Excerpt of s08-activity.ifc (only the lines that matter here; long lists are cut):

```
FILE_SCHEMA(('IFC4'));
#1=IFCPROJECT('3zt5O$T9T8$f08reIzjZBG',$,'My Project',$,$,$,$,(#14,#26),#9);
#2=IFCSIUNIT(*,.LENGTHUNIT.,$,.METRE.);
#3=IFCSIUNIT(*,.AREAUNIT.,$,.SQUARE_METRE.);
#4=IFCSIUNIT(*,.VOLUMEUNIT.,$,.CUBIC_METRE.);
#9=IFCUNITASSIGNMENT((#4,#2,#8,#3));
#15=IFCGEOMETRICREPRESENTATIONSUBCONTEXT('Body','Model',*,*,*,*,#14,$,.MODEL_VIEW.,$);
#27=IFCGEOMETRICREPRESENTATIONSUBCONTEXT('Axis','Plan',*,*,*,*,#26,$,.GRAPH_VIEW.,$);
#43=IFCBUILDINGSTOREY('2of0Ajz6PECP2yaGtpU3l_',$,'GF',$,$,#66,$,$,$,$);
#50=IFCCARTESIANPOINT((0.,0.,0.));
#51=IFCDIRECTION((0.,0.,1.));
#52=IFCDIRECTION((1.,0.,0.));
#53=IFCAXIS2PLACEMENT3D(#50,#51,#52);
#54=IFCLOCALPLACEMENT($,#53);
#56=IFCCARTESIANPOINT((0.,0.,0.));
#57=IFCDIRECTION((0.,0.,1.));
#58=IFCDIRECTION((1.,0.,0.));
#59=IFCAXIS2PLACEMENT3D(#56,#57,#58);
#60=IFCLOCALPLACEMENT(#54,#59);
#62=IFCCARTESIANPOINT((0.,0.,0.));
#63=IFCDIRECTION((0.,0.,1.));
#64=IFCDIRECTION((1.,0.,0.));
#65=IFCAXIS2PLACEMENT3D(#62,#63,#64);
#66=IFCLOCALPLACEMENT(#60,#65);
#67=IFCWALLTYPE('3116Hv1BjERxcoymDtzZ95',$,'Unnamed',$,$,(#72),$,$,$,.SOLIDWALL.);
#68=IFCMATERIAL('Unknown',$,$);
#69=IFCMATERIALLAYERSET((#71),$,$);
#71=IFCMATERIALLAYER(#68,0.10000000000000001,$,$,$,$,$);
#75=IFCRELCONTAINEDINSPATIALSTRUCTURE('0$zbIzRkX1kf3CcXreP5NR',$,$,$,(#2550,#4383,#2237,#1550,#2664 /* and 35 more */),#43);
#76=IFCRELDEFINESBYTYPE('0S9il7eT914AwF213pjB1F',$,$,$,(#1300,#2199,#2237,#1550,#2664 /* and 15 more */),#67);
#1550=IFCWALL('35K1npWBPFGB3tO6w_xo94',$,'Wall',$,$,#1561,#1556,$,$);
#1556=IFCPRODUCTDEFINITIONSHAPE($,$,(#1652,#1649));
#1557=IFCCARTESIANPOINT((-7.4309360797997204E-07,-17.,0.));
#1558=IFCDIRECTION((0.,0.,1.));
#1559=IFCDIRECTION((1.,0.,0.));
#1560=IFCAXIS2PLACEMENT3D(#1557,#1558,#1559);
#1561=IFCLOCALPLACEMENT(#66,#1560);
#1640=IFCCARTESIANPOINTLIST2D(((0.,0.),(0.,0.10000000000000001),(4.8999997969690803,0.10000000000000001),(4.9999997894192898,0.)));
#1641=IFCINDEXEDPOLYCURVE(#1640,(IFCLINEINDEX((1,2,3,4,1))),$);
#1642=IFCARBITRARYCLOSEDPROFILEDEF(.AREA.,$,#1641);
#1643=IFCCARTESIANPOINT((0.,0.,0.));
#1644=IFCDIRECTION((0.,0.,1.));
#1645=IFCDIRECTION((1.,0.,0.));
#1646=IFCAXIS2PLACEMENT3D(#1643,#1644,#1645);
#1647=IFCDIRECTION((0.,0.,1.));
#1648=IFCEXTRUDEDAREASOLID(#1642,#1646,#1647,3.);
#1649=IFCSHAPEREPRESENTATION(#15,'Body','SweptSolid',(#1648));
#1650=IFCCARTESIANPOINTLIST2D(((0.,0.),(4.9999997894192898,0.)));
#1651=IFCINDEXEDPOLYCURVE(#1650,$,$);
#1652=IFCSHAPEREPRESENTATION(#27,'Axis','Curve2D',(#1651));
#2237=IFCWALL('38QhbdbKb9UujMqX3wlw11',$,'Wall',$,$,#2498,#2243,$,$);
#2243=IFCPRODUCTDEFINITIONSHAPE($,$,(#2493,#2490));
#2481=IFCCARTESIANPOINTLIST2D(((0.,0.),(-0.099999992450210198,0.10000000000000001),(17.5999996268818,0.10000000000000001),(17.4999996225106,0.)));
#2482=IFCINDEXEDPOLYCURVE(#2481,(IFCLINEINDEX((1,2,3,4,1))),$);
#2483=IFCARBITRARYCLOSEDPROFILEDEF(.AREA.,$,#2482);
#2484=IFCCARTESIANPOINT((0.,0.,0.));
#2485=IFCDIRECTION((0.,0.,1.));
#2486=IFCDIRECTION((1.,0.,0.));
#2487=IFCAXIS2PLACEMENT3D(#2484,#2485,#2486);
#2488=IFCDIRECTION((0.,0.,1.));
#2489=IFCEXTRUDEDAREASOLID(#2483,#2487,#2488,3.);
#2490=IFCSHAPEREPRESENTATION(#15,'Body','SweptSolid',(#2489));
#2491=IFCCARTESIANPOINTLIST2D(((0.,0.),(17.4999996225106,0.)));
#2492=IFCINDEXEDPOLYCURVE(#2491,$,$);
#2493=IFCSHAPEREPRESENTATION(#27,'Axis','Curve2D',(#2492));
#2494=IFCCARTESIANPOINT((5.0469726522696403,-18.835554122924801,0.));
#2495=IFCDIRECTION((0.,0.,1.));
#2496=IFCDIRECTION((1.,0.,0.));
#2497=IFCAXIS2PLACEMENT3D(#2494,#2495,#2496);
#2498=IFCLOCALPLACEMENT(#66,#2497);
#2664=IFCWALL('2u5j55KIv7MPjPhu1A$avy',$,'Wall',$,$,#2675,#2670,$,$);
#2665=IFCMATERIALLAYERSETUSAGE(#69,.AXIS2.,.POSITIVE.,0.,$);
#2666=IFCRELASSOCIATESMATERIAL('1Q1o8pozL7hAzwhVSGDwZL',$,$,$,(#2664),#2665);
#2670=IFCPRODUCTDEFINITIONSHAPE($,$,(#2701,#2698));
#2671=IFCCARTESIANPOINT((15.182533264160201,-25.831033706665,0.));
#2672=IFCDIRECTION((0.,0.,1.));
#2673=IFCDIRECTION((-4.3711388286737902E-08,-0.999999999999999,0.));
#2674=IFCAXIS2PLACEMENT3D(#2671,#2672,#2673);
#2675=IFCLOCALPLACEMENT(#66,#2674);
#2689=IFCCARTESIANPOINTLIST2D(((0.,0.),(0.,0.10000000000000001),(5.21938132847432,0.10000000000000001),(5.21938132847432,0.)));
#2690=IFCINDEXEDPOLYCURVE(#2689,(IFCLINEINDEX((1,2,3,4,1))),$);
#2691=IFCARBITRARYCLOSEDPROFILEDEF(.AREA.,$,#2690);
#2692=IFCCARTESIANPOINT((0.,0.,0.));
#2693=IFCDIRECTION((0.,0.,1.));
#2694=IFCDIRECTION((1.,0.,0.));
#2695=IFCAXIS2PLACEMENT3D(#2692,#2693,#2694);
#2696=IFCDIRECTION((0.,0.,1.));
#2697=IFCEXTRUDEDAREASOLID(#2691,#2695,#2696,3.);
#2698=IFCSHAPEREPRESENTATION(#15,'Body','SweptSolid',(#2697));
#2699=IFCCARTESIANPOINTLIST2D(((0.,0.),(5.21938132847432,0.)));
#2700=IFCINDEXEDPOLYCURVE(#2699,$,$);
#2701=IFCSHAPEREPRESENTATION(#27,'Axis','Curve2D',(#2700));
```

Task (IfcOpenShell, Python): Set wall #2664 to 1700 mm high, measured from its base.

```python
import ifcopenshell
import ifcopenshell.geom
import ifcopenshell.util.representation
import ifcopenshell.util.shape
import ifcopenshell.util.unit

model = ifcopenshell.open("s08-activity.ifc")
unit_scale = ifcopenshell.util.unit.calculate_unit_scale(model)
settings = ifcopenshell.geom.settings()


def volume(element):
    """Net volume in cubic metres, openings subtracted."""
    shape = ifcopenshell.geom.create_shape(settings, element)
    return ifcopenshell.util.shape.get_volume(shape.geometry)


wall = model.by_guid("2u5j55KIv7MPjPhu1A$avy")
before = volume(wall)

body = ifcopenshell.util.representation.get_representation(wall, "Model", "Body")
solid = body.Items[0]
old_height = solid.Depth
solid.Depth = 1.7 / unit_scale
after = volume(wall)

print(f"height {old_height:g} -> {solid.Depth:g}, volume {before:.3f} -> {after:.3f} m3")

model.write("s08-activity_rev.ifc")
```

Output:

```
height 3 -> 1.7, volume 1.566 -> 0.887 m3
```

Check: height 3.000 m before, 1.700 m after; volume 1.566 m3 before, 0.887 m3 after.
